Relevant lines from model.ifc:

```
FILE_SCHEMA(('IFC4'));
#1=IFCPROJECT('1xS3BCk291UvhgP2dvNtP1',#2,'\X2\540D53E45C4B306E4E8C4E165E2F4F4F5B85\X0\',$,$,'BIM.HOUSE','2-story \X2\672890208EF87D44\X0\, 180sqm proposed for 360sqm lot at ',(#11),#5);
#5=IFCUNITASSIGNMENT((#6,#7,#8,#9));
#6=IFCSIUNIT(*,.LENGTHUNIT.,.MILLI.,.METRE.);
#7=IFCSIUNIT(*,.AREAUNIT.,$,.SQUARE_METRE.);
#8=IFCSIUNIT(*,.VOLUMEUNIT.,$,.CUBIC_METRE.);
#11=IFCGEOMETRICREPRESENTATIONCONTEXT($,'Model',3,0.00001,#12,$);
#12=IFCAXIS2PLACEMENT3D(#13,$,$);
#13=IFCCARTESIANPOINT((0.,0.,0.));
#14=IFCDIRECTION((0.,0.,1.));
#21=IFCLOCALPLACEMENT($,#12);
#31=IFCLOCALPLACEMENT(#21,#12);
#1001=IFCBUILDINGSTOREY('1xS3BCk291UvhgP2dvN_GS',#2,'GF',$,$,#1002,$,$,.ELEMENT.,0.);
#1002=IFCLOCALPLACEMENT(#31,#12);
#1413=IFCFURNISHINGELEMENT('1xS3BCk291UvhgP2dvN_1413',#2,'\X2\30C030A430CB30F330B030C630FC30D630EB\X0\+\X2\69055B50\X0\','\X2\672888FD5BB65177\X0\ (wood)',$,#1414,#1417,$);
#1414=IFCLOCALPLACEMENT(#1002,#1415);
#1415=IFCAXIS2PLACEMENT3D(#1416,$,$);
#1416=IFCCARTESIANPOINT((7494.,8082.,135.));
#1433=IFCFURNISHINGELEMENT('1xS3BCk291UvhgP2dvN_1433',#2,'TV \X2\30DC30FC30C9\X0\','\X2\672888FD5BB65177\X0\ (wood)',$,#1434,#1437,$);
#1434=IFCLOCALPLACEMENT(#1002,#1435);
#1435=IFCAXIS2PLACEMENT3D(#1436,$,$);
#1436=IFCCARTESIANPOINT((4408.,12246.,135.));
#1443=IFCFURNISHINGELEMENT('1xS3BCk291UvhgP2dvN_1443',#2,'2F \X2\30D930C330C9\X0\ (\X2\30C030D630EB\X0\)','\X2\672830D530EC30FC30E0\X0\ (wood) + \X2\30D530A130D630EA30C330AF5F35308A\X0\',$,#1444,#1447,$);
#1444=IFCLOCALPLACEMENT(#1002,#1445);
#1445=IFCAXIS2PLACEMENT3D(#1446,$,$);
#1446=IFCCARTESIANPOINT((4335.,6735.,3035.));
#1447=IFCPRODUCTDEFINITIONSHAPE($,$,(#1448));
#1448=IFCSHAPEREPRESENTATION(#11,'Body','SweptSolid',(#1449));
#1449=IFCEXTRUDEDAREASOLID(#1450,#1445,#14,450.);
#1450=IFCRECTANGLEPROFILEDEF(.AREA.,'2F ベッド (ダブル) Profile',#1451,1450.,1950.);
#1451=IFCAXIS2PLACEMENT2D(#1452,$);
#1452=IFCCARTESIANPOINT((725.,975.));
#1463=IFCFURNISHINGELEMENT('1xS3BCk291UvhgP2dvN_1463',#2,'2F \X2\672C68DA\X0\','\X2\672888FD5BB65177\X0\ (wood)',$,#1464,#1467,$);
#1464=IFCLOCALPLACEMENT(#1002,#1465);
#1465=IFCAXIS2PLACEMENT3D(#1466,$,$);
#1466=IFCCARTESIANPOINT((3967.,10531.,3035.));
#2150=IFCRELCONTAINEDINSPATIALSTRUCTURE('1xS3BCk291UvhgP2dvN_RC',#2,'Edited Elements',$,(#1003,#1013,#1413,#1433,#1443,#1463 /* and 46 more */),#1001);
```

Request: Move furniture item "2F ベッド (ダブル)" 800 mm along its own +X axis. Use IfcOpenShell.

```python
import ifcopenshell
import ifcopenshell.api.geometry
import ifcopenshell.util.placement
import ifcopenshell.util.unit

model = ifcopenshell.open("model.ifc")
unit_scale = ifcopenshell.util.unit.calculate_unit_scale(model)

item = model.by_guid("1xS3BCk291UvhgP2dvN_1443")
matrix = ifcopenshell.util.placement.get_local_placement(item.ObjectPlacement)
matrix[:3, 3] += matrix[:3, 0] * 0.8 / unit_scale
ifcopenshell.api.geometry.edit_object_placement(model, product=item, matrix=matrix, is_si=False)

print(ifcopenshell.util.placement.get_local_placement(item.ObjectPlacement).round(3) + 0.0)

model.write("model-out.ifc")
```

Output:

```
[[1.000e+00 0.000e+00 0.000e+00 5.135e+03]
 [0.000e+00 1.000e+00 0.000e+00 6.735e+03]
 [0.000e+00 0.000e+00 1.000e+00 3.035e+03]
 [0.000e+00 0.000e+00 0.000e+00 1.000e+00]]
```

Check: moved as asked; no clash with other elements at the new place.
